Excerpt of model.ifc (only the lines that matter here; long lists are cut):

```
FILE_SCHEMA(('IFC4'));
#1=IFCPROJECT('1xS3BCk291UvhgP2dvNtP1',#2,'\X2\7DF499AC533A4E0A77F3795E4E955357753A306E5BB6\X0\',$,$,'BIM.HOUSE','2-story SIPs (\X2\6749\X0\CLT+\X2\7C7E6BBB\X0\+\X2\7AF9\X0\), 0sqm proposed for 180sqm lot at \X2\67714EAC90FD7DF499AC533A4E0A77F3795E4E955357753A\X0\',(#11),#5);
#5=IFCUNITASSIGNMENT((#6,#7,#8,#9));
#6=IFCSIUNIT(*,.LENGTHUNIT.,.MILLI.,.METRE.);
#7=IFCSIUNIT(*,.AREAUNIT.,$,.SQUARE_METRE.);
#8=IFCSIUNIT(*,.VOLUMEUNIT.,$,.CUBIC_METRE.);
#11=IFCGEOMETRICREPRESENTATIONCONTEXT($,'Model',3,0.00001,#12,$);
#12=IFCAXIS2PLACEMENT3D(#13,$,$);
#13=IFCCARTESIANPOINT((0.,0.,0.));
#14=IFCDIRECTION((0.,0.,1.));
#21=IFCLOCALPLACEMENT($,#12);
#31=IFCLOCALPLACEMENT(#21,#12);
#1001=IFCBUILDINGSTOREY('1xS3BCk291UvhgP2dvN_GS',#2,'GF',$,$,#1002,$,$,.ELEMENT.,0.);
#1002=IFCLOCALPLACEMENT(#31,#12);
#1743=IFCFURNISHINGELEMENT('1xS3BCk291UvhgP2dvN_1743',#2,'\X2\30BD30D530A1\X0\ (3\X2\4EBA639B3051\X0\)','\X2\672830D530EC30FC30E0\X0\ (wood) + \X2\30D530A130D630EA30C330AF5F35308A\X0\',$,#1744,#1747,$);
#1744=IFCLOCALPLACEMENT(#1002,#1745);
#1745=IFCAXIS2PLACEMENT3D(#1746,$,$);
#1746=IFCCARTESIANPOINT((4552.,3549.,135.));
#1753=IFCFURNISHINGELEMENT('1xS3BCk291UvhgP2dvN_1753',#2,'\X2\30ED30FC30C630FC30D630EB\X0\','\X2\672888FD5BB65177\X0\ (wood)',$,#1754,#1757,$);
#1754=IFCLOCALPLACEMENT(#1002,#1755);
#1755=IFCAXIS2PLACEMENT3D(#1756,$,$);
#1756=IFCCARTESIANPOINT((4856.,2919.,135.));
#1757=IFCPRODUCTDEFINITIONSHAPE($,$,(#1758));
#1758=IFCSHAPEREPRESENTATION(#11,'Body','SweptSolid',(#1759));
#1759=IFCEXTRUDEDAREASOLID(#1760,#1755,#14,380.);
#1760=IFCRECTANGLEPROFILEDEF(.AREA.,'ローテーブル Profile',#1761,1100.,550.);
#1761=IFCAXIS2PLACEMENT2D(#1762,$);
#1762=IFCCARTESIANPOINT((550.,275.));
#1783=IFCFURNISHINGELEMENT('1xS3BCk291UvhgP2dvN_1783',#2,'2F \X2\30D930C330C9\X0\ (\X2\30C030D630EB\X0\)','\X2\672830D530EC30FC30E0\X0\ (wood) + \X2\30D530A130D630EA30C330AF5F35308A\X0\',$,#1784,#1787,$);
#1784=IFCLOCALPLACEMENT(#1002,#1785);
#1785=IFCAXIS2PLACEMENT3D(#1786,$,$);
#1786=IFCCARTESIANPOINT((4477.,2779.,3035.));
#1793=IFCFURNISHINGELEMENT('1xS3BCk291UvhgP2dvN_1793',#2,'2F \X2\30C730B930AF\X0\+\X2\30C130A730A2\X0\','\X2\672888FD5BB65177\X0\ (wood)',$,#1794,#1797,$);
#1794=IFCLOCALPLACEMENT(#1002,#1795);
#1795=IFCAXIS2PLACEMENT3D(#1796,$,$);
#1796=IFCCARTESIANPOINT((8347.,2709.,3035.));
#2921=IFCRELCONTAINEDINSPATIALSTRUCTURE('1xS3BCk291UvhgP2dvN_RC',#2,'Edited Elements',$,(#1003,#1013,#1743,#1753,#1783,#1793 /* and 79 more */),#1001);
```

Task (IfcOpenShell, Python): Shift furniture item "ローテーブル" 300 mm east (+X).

```python
import ifcopenshell
import ifcopenshell.api.geometry
import ifcopenshell.util.placement
import ifcopenshell.util.unit

model = ifcopenshell.open("model.ifc")
unit_scale = ifcopenshell.util.unit.calculate_unit_scale(model)

item = model.by_id(1753)
matrix = ifcopenshell.util.placement.get_local_placement(item.ObjectPlacement)
matrix[0, 3] += 0.3 / unit_scale
ifcopenshell.api.geometry.edit_object_placement(model, product=item, matrix=matrix, is_si=False)

print(ifcopenshell.util.placement.get_local_placement(item.ObjectPlacement).round(3) + 0.0)

model.write("model_edited.ifc")
```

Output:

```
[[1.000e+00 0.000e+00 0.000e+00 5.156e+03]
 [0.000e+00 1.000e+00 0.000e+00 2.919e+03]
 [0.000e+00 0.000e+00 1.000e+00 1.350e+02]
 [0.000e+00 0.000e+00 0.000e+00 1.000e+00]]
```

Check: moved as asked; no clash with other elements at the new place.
